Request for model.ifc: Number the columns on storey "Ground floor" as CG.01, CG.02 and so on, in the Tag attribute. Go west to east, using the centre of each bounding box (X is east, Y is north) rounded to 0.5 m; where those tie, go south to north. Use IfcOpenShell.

First a look at what the model holds.

```python
import ifcopenshell
import ifcopenshell.util.element
import ifcopenshell.util.placement

model = ifcopenshell.open("model.ifc")
print(model.schema)
storey = next(s for s in model.by_type("IfcBuildingStorey") if s.Name == "Ground floor")
columns = [e for e in ifcopenshell.util.element.get_decomposition(storey) if e.is_a("IfcColumn")]
for e in sorted(columns, key=lambda e: e.id()):
    origin = ifcopenshell.util.placement.get_local_placement(e.ObjectPlacement)[:3, 3]
    print(e.id(), e.Tag, e.Name, origin.round(2) + 0.0, sep=" | ")
```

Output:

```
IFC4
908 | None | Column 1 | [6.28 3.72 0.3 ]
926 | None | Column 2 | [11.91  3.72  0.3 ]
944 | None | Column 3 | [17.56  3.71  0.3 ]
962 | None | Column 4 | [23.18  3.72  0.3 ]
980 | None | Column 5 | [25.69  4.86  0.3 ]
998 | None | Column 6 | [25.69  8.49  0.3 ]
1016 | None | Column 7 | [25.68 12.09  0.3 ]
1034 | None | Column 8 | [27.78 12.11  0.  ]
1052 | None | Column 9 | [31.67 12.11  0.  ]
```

```python
import ifcopenshell
import ifcopenshell.geom
import ifcopenshell.util.element
import ifcopenshell.util.shape

model = ifcopenshell.open("model.ifc")
settings = ifcopenshell.geom.settings()
settings.set("use-world-coords", True)


def centre(element):
    shape = ifcopenshell.geom.create_shape(settings, element)
    return ifcopenshell.util.shape.get_bbox_centroid(shape.geometry)


storey = next(s for s in model.by_type("IfcBuildingStorey") if s.Name == "Ground floor")
columns = [e for e in ifcopenshell.util.element.get_decomposition(storey) if e.is_a("IfcColumn")]

# Insertion points can sit at a corner or the storey origin, so sort by the geometry (in metres).
centres = {e: centre(e) for e in columns}
columns.sort(key=lambda e: (round(centres[e][0] / 0.5), centres[e][1]))

for i, e in enumerate(columns, start=1):
    number = f"CG.{i:02d}"
    e.Tag = number
    print(e.id(), number)

model.write("model_v2.ifc")
```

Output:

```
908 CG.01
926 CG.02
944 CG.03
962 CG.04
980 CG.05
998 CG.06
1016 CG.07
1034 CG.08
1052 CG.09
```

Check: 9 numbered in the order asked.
